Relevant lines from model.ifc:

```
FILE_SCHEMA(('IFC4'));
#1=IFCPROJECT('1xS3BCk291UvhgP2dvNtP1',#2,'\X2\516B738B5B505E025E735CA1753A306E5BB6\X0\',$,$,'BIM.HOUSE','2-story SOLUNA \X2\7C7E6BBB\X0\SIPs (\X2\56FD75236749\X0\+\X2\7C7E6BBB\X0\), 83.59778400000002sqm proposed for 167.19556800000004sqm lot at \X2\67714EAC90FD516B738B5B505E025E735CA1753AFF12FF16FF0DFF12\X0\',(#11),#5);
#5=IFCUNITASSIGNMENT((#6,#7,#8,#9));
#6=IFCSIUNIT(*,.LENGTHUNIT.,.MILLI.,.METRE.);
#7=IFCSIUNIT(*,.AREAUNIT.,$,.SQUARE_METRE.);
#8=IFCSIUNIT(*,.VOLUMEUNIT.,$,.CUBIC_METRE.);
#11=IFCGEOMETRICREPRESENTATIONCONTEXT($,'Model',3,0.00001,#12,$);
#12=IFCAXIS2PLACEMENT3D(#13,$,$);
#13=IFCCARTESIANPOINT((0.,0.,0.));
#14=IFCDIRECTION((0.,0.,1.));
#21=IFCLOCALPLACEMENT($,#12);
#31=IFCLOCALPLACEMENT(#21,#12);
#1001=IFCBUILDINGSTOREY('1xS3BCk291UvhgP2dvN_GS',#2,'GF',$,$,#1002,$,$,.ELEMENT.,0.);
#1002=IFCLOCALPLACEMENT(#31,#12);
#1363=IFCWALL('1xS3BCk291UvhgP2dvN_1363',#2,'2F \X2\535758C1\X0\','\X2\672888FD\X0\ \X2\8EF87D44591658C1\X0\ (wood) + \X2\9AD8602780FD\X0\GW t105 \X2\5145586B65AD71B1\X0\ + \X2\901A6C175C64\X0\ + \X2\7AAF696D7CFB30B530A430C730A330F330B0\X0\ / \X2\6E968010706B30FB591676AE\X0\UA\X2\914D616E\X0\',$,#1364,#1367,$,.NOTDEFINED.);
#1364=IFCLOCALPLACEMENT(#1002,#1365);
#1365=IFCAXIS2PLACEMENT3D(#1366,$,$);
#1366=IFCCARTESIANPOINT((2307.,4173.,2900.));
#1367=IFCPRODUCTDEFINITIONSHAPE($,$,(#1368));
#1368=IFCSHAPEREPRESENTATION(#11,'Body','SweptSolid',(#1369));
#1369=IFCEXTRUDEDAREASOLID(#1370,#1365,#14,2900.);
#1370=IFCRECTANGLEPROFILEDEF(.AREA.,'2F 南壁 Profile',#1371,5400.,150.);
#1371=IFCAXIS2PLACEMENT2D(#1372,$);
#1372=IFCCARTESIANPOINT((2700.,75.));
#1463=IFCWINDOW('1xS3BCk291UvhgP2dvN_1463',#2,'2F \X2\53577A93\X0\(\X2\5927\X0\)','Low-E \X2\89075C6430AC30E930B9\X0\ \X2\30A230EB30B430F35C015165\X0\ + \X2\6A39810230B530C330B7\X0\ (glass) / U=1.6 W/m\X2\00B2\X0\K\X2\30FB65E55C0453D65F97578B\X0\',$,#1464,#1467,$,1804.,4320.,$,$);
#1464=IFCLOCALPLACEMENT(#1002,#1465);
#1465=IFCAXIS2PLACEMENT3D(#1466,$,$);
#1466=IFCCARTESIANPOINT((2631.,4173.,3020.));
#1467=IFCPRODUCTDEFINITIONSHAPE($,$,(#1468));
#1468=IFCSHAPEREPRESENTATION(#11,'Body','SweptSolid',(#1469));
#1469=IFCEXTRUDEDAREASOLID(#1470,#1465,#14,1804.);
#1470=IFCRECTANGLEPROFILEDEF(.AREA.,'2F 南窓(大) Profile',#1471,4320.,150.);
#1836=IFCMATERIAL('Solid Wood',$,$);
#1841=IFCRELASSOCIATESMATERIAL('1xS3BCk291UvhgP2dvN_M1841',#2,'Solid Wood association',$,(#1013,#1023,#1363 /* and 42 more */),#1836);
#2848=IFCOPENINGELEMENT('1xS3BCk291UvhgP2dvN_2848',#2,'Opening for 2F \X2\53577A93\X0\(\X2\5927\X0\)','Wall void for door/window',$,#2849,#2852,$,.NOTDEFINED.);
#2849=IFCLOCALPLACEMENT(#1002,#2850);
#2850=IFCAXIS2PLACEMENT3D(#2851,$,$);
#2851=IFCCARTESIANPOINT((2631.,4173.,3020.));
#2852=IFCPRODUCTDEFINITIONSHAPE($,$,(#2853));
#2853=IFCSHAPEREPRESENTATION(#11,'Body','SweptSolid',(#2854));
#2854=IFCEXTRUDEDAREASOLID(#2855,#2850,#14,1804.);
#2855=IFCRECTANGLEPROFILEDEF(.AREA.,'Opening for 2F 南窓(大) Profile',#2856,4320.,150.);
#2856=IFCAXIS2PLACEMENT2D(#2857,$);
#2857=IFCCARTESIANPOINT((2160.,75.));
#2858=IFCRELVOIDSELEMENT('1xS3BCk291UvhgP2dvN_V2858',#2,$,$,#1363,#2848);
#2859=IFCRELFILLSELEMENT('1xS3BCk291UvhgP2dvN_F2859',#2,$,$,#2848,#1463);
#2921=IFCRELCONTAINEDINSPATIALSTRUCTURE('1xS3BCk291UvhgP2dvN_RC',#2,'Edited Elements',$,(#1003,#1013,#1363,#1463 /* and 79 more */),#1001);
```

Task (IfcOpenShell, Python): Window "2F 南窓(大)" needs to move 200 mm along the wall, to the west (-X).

```python
import ifcopenshell
import ifcopenshell.api.geometry
import ifcopenshell.util.placement
import ifcopenshell.util.unit

model = ifcopenshell.open("model.ifc")
unit_scale = ifcopenshell.util.unit.calculate_unit_scale(model)

window = model.by_guid("1xS3BCk291UvhgP2dvN_1463")
opening = window.FillsVoids[0].RelatingOpeningElement
wall = opening.VoidsElements[0].RelatingBuildingElement

wall_matrix = ifcopenshell.util.placement.get_local_placement(wall.ObjectPlacement)
shift = wall_matrix[:3, 0] * -0.2 / unit_scale
before = ifcopenshell.util.placement.get_local_placement(window.ObjectPlacement)[:3, 3].copy()

# The window is not placed relative to its opening, so move both.
for product in (opening, window):
    matrix = ifcopenshell.util.placement.get_local_placement(product.ObjectPlacement)
    matrix[:3, 3] += shift
    ifcopenshell.api.geometry.edit_object_placement(model, product=product, matrix=matrix, is_si=False)

after = ifcopenshell.util.placement.get_local_placement(window.ObjectPlacement)[:3, 3]
print("window moved by", (after - before).round(3) + 0.0)

model.write("model_rev.ifc")
```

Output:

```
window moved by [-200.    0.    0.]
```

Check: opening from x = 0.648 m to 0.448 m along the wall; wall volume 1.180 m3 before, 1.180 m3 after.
